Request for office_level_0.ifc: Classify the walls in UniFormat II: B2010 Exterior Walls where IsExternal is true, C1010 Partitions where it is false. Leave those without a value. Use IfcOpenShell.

First a look at what the model holds.

```python
import ifcopenshell
import ifcopenshell.util.element

model = ifcopenshell.open("office_level_0.ifc")
print(model.schema)
print("classifications:", [c.Name for c in model.by_type("IfcClassification")])
values = [ifcopenshell.util.element.get_pset(e, "Pset_WallCommon", "IsExternal") for e in model.by_type("IfcWall")]
for value in (True, False, None):
    print("IsExternal", value, values.count(value))
```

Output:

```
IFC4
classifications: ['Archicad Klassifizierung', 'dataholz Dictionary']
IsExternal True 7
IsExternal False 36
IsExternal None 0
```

```python
import ifcopenshell
import ifcopenshell.api.classification
import ifcopenshell.util.element

model = ifcopenshell.open("office_level_0.ifc")

system = ifcopenshell.api.classification.add_classification(model, classification="UniFormat II")

walls = model.by_type("IfcWall")
external = {e: ifcopenshell.util.element.get_pset(e, "Pset_WallCommon", "IsExternal") for e in walls}
for flag, code, name in ((True, "B2010", "Exterior Walls"), (False, "C1010", "Partitions")):
    products = [e for e in walls if external[e] is flag]
    ifcopenshell.api.classification.add_reference(
        model, products=products, classification=system, identification=code, name=name
    )
    print(code, len(products))

model.write("office_level_0_edited.ifc")
```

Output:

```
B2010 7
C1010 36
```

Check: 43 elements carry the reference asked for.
